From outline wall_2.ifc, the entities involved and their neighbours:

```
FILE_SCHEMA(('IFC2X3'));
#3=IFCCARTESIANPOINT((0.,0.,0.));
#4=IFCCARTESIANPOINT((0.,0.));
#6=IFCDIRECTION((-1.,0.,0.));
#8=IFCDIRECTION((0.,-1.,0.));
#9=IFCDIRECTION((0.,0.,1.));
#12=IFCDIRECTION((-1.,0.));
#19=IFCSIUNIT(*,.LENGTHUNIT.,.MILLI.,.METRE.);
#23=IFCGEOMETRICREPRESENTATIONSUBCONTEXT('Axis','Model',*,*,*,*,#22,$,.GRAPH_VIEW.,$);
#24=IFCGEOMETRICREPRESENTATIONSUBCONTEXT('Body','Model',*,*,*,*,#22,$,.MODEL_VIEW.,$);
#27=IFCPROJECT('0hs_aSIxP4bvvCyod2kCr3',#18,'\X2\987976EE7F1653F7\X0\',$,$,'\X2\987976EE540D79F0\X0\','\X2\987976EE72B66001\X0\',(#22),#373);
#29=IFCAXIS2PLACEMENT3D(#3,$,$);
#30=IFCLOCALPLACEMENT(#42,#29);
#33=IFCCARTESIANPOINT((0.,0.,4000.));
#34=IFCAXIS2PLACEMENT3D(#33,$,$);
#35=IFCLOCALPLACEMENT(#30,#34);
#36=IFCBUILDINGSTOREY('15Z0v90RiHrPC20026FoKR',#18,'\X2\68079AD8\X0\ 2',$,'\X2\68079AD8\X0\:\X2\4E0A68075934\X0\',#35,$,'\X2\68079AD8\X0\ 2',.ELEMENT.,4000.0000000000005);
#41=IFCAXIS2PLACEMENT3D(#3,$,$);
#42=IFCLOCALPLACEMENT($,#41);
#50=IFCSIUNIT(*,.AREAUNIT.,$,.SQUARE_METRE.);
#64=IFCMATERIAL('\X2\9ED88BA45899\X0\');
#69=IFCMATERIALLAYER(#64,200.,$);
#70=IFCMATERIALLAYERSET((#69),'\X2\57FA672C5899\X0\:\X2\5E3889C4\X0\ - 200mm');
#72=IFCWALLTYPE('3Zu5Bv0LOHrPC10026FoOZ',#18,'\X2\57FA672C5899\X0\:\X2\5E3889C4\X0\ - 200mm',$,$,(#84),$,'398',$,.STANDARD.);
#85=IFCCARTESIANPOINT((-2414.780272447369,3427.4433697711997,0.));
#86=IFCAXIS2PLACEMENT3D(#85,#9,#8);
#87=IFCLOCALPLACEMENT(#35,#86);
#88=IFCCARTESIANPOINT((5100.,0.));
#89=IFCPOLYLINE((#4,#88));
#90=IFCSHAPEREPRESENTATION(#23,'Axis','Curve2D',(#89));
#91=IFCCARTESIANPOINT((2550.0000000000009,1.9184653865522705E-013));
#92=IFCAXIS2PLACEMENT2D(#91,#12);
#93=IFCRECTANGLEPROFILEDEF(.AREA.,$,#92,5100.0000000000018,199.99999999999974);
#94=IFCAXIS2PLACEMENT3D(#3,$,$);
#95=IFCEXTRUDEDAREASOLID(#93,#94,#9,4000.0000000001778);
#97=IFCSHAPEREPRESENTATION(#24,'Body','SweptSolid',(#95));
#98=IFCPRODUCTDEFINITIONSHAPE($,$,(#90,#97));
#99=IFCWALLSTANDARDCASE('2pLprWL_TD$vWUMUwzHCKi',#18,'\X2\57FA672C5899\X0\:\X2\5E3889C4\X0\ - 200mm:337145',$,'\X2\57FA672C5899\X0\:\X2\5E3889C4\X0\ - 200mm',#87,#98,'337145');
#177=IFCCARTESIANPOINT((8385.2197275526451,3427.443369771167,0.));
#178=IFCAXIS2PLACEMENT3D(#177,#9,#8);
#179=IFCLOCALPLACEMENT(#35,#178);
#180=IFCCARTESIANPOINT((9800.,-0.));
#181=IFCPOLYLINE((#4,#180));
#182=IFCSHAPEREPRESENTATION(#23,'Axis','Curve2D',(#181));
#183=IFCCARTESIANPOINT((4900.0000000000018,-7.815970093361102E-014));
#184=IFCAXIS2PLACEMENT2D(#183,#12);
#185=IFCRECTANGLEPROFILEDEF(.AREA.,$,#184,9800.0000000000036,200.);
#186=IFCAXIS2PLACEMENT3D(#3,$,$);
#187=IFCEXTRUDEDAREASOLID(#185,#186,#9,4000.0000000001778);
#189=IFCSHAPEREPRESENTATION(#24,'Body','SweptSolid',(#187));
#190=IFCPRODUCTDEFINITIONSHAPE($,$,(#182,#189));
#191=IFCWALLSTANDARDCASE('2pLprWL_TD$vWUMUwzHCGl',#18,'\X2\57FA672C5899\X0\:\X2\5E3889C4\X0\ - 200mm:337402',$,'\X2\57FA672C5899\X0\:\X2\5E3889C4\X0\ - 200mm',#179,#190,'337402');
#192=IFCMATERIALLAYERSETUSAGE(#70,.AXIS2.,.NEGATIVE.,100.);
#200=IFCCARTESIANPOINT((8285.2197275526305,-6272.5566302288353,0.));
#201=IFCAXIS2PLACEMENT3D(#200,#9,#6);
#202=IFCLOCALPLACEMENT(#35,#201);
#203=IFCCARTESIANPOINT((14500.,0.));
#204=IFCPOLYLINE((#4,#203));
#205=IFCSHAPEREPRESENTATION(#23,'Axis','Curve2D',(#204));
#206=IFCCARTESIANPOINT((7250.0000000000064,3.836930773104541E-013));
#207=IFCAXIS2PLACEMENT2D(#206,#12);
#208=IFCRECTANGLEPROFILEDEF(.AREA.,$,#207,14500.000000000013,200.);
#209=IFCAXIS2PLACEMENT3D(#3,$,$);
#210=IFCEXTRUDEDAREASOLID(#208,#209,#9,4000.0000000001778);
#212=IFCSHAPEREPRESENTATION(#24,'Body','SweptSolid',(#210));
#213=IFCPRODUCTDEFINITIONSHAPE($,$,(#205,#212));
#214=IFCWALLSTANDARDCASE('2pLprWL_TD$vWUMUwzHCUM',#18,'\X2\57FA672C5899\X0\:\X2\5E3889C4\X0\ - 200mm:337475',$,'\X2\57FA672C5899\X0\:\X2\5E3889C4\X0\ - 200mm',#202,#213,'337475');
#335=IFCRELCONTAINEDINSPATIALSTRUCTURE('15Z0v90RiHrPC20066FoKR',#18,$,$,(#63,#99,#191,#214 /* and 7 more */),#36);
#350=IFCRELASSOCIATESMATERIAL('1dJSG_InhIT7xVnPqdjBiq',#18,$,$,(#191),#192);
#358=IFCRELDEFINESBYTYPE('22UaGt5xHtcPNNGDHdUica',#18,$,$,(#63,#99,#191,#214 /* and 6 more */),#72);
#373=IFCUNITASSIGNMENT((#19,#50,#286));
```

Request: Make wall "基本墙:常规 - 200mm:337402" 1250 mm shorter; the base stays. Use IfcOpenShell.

```python
import ifcopenshell
import ifcopenshell.geom
import ifcopenshell.util.representation
import ifcopenshell.util.shape

model = ifcopenshell.open("outline wall_2.ifc")
settings = ifcopenshell.geom.settings()


def volume(element):
    """Net volume in cubic metres, openings subtracted."""
    shape = ifcopenshell.geom.create_shape(settings, element)
    return ifcopenshell.util.shape.get_volume(shape.geometry)


wall = model.by_id(191)
before = volume(wall)

body = ifcopenshell.util.representation.get_representation(wall, "Model", "Body")
solid = body.Items[0]
old_height = solid.Depth
solid.Depth -= 1250.0
after = volume(wall)

print(f"height {old_height:g} -> {solid.Depth:g}, volume {before:.3f} -> {after:.3f} m3")

model.write("outline wall_2_updated.ifc")
```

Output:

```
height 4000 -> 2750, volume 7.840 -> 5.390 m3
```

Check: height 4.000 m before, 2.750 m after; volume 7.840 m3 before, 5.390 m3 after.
